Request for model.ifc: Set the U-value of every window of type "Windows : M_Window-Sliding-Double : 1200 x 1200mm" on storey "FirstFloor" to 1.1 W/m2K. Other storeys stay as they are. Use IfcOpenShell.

First a look at what the model holds.

```python
import ifcopenshell
import ifcopenshell.util.element

model = ifcopenshell.open("model.ifc")
print(model.schema)
storey = next(s for s in model.by_type("IfcBuildingStorey") if s.Name == "FirstFloor")
windows = [e for e in ifcopenshell.util.element.get_decomposition(storey) if e.is_a("IfcWindow")]
seen = {}
for e in windows:
    element_type = ifcopenshell.util.element.get_type(e)
    key = (element_type.Name if element_type != e and element_type else None, ifcopenshell.util.element.get_pset(e, "Pset_WindowCommon", "ThermalTransmittance"))
    seen[key] = seen.get(key, 0) + 1
for (name, value), count in sorted(seen.items(), key=str):
    print(count, "x", name, "|", value)
```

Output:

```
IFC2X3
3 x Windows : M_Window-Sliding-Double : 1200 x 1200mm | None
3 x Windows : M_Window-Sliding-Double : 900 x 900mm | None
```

```python
import ifcopenshell
import ifcopenshell.api.pset
import ifcopenshell.util.element

model = ifcopenshell.open("model.ifc")

storey = next(s for s in model.by_type("IfcBuildingStorey") if s.Name == "FirstFloor")
windows = [e for e in ifcopenshell.util.element.get_decomposition(storey) if e.is_a("IfcWindow")]

count = 0
for e in windows:
    element_type = ifcopenshell.util.element.get_type(e)
    if element_type in (None, e) or element_type.Name != "Windows : M_Window-Sliding-Double : 1200 x 1200mm":
        continue
    # add_pset returns the element's existing set when there is one.
    pset = ifcopenshell.api.pset.add_pset(model, product=e, name="Pset_WindowCommon")
    ifcopenshell.api.pset.edit_pset(model, pset=pset, properties={"ThermalTransmittance": 1.1})
    count += 1

print(count, "windows updated")

model.write("model_edited.ifc")
```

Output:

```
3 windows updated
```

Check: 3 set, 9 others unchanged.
